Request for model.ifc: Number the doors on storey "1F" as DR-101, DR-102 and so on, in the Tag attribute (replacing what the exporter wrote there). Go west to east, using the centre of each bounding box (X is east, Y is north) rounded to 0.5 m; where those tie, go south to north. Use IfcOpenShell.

First a look at what the model holds.

```python
import ifcopenshell
import ifcopenshell.util.element
import ifcopenshell.util.placement

model = ifcopenshell.open("model.ifc")
print(model.schema)
storey = next(s for s in model.by_type("IfcBuildingStorey") if s.Name == "1F")
doors = [e for e in ifcopenshell.util.element.get_decomposition(storey) if e.is_a("IfcDoor")]
for e in sorted(doors, key=lambda e: e.id()):
    origin = ifcopenshell.util.placement.get_local_placement(e.ObjectPlacement)[:3, 3]
    print(e.id(), e.Tag, e.Name, origin.round(2) + 0.0, sep=" | ")
```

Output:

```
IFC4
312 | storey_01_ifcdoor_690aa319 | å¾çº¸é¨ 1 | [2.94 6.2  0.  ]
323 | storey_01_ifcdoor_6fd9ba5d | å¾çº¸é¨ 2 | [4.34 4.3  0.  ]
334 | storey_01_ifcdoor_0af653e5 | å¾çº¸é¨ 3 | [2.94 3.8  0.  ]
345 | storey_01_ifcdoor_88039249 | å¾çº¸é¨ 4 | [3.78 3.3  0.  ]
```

```python
import ifcopenshell
import ifcopenshell.geom
import ifcopenshell.util.element
import ifcopenshell.util.shape

model = ifcopenshell.open("model.ifc")
settings = ifcopenshell.geom.settings()
settings.set("use-world-coords", True)


def centre(element):
    shape = ifcopenshell.geom.create_shape(settings, element)
    return ifcopenshell.util.shape.get_bbox_centroid(shape.geometry)


storey = next(s for s in model.by_type("IfcBuildingStorey") if s.Name == "1F")
doors = [e for e in ifcopenshell.util.element.get_decomposition(storey) if e.is_a("IfcDoor")]

# Insertion points can sit at a corner or the storey origin, so sort by the geometry (in metres).
centres = {e: centre(e) for e in doors}
doors.sort(key=lambda e: (round(centres[e][0] / 0.5), centres[e][1]))

for i, e in enumerate(doors, start=1):
    number = f"DR-1{i:02d}"
    e.Tag = number
    print(e.id(), number)

model.write("model-out.ifc")
```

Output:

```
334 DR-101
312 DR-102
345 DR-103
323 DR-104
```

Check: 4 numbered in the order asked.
